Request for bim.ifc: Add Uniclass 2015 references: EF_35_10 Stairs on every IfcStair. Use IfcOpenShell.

First a look at what the model holds.

```python
import ifcopenshell

model = ifcopenshell.open("bim.ifc")
print(model.schema)
print("classifications:", [c.Name for c in model.by_type("IfcClassification")])
for ifc_class in ("IfcDoor", "IfcRoof", "IfcStair", "IfcWall", "IfcWindow"):
    print(ifc_class, len(model.by_type(ifc_class)))
```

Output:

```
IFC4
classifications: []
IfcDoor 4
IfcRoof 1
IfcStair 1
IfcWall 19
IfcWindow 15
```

```python
import ifcopenshell
import ifcopenshell.api.classification

model = ifcopenshell.open("bim.ifc")

system = ifcopenshell.api.classification.add_classification(model, classification="Uniclass 2015")

codes = {
    "IfcStair": ("EF_35_10", "Stairs"),
}
for ifc_class, (code, name) in codes.items():
    products = model.by_type(ifc_class)
    ifcopenshell.api.classification.add_reference(
        model, products=products, classification=system, identification=code, name=name
    )
    print(code, len(products))

model.write("bim_updated.ifc")
```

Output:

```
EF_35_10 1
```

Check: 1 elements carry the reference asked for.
